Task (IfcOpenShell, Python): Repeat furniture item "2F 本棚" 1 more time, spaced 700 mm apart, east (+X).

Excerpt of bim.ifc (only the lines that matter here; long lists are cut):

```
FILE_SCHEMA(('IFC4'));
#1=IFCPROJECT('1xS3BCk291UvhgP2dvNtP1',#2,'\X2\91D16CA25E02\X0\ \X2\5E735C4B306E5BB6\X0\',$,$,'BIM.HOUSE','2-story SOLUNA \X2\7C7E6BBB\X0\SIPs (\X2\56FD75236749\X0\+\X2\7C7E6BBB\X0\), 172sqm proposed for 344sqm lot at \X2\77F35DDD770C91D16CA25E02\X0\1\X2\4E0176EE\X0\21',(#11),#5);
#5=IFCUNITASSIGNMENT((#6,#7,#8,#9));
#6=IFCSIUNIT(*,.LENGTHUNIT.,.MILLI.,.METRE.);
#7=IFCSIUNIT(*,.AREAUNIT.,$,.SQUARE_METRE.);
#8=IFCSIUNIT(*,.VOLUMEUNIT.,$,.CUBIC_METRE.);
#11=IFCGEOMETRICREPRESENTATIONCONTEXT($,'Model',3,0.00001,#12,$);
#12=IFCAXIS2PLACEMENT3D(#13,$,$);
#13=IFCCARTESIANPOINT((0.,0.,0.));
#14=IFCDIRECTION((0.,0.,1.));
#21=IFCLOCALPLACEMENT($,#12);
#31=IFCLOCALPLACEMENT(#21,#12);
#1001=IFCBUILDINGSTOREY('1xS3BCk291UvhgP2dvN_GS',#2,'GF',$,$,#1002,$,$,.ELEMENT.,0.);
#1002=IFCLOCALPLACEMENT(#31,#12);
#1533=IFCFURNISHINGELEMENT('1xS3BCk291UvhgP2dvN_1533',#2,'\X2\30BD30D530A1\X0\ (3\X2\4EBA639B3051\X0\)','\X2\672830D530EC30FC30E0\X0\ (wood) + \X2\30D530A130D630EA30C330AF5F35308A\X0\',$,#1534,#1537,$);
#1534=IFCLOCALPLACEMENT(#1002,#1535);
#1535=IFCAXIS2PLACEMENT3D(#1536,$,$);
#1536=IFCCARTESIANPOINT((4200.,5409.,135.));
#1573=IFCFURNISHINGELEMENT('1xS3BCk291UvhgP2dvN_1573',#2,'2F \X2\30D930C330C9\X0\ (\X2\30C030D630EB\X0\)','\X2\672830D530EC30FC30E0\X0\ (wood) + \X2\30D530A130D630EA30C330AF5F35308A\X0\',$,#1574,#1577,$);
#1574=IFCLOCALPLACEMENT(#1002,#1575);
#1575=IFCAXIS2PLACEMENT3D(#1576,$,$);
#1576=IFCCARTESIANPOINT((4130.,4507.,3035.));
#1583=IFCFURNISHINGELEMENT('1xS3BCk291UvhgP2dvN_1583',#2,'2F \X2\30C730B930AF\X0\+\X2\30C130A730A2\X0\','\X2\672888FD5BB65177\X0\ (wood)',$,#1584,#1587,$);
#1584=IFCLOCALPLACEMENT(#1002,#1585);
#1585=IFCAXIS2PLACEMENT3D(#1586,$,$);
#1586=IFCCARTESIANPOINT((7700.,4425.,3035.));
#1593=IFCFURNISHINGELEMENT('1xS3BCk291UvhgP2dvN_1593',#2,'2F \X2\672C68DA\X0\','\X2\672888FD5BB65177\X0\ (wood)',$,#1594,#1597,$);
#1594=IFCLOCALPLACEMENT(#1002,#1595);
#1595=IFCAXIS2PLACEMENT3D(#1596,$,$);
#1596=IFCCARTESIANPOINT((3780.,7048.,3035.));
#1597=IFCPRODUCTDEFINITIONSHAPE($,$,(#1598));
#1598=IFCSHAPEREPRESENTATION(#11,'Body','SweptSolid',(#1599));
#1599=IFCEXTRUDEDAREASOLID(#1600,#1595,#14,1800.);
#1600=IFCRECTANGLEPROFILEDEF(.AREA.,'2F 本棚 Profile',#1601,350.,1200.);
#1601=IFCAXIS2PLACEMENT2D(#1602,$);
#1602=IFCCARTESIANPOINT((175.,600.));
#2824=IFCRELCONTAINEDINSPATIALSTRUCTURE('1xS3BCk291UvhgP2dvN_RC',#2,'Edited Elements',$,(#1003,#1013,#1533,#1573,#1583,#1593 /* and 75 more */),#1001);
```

```python
import numpy as np
import ifcopenshell
import ifcopenshell.api.geometry
import ifcopenshell.api.root
import ifcopenshell.util.element
import ifcopenshell.util.placement
import ifcopenshell.util.unit

model = ifcopenshell.open("bim.ifc")
unit_scale = ifcopenshell.util.unit.calculate_unit_scale(model)


def reuse_history(source, copy):
    """copy_class also copies each property set's owner history, people and application; keep the originals."""
    for rel in copy.IsDefinedBy:
        if rel.is_a("IfcRelDefinesByProperties") and (history := rel.RelatingPropertyDefinition.OwnerHistory):
            rel.RelatingPropertyDefinition.OwnerHistory = source.OwnerHistory
            ifcopenshell.util.element.remove_deep2(model, history)


source = model.by_guid("1xS3BCk291UvhgP2dvN_1593")
base = ifcopenshell.util.placement.get_local_placement(source.ObjectPlacement)
step = np.array([1.0, 0.0, 0.0]) * 0.7 / unit_scale

for i in range(1, 2):
    copy = ifcopenshell.api.root.copy_class(model, product=source)
    copy.Representation = ifcopenshell.util.element.copy_deep(
        model, source.Representation, exclude=["IfcGeometricRepresentationContext", "IfcRepresentationMap"]
    )
    reuse_history(source, copy)
    matrix = base.copy()
    matrix[:3, 3] += i * step
    print("added at", matrix[:3, 3].round(3) + 0.0)
    ifcopenshell.api.geometry.edit_object_placement(model, product=copy, matrix=matrix, is_si=False)

model.write("bim_rev.ifc")
```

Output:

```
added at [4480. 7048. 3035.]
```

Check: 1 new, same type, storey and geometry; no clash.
